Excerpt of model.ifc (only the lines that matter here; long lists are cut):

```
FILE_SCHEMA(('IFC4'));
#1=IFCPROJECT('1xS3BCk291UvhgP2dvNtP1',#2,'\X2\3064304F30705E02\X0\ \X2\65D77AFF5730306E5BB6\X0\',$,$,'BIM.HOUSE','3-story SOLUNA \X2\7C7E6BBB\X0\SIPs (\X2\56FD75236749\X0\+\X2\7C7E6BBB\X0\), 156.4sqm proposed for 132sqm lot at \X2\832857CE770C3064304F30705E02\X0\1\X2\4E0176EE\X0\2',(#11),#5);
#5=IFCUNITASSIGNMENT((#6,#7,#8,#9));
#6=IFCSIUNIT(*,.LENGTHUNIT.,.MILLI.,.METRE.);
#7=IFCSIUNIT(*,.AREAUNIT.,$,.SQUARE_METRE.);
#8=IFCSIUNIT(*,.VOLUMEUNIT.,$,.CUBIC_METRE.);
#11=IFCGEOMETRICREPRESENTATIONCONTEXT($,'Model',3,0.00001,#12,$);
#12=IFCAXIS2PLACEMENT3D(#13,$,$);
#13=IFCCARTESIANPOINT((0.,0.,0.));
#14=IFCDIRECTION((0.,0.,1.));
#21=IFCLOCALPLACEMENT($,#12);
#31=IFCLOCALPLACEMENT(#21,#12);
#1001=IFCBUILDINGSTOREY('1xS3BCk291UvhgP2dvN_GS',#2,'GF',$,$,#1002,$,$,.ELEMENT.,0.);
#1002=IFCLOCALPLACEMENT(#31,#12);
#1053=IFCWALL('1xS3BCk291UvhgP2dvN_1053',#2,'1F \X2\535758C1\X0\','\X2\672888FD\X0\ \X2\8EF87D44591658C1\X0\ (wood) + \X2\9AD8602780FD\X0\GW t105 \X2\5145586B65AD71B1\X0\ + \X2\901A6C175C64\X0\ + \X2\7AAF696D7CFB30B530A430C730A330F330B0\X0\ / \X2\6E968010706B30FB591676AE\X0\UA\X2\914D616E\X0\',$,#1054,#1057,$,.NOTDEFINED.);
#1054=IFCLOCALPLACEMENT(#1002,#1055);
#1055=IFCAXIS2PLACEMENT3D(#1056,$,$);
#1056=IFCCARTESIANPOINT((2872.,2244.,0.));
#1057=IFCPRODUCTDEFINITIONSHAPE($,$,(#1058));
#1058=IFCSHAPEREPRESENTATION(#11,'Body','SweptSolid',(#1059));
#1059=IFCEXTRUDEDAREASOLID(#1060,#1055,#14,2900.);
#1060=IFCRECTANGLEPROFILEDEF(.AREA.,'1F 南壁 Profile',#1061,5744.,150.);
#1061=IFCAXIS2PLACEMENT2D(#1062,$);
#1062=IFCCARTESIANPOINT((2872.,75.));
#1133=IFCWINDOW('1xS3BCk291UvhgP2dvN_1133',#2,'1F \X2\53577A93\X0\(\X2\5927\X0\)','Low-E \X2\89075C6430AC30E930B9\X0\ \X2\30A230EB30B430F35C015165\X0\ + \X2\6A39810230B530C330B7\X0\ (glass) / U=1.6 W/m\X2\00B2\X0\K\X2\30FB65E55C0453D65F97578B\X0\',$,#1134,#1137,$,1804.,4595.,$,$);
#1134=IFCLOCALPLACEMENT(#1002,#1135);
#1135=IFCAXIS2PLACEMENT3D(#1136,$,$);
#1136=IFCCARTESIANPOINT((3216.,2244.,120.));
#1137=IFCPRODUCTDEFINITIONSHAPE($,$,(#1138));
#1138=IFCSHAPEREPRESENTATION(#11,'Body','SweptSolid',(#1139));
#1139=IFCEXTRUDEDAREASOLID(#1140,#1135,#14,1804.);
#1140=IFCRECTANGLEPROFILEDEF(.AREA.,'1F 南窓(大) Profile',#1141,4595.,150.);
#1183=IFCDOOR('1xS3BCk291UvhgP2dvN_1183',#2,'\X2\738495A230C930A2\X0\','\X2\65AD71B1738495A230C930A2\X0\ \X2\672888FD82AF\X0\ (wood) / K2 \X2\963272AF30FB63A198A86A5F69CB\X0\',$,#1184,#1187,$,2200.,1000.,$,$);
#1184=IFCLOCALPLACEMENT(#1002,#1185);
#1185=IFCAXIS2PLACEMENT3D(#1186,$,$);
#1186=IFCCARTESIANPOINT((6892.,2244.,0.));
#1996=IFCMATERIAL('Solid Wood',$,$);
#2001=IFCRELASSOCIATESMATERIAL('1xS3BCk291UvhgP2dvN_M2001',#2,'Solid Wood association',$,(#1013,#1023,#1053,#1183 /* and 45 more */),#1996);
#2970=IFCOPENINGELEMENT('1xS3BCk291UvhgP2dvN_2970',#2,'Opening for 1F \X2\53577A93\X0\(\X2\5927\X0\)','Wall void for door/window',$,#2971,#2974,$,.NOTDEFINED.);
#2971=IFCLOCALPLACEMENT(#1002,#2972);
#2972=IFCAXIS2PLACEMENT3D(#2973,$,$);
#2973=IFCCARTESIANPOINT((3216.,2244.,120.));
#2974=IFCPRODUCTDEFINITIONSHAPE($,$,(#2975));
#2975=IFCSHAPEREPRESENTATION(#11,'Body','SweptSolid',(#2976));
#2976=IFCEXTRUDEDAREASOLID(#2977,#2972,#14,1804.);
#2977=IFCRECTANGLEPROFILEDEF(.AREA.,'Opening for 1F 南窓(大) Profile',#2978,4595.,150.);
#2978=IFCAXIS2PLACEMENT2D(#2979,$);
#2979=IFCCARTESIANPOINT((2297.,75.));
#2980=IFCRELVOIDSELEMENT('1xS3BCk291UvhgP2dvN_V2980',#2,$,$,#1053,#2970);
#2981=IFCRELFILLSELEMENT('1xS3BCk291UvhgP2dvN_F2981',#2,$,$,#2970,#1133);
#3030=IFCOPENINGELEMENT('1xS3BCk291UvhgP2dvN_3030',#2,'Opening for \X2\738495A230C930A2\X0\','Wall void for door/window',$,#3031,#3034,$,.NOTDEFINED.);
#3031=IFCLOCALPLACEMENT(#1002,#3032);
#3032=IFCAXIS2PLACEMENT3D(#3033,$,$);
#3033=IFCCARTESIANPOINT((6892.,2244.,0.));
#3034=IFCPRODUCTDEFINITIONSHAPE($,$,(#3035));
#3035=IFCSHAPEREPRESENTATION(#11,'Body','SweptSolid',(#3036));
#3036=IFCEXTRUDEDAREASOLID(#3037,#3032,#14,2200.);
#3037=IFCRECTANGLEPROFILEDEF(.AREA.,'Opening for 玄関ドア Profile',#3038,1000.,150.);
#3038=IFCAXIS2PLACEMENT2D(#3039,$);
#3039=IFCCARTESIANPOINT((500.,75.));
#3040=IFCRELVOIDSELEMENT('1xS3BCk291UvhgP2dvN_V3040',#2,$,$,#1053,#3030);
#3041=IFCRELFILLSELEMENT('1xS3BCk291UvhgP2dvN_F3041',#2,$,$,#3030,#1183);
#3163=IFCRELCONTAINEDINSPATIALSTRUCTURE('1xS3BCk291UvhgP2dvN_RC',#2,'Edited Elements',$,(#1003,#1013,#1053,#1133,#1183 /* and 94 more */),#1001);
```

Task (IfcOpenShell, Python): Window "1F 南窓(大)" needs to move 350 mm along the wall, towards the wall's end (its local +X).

```python
import ifcopenshell
import ifcopenshell.api.geometry
import ifcopenshell.util.placement

model = ifcopenshell.open("model.ifc")

window = model.by_guid("1xS3BCk291UvhgP2dvN_1133")
opening = window.FillsVoids[0].RelatingOpeningElement
wall = opening.VoidsElements[0].RelatingBuildingElement

wall_matrix = ifcopenshell.util.placement.get_local_placement(wall.ObjectPlacement)
shift = wall_matrix[:3, 0] * 350.0
before = ifcopenshell.util.placement.get_local_placement(window.ObjectPlacement)[:3, 3].copy()

# The window is not placed relative to its opening, so move both.
for product in (opening, window):
    matrix = ifcopenshell.util.placement.get_local_placement(product.ObjectPlacement)
    matrix[:3, 3] += shift
    ifcopenshell.api.geometry.edit_object_placement(model, product=product, matrix=matrix, is_si=False)

after = ifcopenshell.util.placement.get_local_placement(window.ObjectPlacement)[:3, 3]
print("window moved by", (after - before).round(3) + 0.0)

model.write("model_rev.ifc")
```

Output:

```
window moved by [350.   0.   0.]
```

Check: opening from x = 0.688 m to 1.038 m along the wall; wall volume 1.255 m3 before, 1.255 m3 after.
